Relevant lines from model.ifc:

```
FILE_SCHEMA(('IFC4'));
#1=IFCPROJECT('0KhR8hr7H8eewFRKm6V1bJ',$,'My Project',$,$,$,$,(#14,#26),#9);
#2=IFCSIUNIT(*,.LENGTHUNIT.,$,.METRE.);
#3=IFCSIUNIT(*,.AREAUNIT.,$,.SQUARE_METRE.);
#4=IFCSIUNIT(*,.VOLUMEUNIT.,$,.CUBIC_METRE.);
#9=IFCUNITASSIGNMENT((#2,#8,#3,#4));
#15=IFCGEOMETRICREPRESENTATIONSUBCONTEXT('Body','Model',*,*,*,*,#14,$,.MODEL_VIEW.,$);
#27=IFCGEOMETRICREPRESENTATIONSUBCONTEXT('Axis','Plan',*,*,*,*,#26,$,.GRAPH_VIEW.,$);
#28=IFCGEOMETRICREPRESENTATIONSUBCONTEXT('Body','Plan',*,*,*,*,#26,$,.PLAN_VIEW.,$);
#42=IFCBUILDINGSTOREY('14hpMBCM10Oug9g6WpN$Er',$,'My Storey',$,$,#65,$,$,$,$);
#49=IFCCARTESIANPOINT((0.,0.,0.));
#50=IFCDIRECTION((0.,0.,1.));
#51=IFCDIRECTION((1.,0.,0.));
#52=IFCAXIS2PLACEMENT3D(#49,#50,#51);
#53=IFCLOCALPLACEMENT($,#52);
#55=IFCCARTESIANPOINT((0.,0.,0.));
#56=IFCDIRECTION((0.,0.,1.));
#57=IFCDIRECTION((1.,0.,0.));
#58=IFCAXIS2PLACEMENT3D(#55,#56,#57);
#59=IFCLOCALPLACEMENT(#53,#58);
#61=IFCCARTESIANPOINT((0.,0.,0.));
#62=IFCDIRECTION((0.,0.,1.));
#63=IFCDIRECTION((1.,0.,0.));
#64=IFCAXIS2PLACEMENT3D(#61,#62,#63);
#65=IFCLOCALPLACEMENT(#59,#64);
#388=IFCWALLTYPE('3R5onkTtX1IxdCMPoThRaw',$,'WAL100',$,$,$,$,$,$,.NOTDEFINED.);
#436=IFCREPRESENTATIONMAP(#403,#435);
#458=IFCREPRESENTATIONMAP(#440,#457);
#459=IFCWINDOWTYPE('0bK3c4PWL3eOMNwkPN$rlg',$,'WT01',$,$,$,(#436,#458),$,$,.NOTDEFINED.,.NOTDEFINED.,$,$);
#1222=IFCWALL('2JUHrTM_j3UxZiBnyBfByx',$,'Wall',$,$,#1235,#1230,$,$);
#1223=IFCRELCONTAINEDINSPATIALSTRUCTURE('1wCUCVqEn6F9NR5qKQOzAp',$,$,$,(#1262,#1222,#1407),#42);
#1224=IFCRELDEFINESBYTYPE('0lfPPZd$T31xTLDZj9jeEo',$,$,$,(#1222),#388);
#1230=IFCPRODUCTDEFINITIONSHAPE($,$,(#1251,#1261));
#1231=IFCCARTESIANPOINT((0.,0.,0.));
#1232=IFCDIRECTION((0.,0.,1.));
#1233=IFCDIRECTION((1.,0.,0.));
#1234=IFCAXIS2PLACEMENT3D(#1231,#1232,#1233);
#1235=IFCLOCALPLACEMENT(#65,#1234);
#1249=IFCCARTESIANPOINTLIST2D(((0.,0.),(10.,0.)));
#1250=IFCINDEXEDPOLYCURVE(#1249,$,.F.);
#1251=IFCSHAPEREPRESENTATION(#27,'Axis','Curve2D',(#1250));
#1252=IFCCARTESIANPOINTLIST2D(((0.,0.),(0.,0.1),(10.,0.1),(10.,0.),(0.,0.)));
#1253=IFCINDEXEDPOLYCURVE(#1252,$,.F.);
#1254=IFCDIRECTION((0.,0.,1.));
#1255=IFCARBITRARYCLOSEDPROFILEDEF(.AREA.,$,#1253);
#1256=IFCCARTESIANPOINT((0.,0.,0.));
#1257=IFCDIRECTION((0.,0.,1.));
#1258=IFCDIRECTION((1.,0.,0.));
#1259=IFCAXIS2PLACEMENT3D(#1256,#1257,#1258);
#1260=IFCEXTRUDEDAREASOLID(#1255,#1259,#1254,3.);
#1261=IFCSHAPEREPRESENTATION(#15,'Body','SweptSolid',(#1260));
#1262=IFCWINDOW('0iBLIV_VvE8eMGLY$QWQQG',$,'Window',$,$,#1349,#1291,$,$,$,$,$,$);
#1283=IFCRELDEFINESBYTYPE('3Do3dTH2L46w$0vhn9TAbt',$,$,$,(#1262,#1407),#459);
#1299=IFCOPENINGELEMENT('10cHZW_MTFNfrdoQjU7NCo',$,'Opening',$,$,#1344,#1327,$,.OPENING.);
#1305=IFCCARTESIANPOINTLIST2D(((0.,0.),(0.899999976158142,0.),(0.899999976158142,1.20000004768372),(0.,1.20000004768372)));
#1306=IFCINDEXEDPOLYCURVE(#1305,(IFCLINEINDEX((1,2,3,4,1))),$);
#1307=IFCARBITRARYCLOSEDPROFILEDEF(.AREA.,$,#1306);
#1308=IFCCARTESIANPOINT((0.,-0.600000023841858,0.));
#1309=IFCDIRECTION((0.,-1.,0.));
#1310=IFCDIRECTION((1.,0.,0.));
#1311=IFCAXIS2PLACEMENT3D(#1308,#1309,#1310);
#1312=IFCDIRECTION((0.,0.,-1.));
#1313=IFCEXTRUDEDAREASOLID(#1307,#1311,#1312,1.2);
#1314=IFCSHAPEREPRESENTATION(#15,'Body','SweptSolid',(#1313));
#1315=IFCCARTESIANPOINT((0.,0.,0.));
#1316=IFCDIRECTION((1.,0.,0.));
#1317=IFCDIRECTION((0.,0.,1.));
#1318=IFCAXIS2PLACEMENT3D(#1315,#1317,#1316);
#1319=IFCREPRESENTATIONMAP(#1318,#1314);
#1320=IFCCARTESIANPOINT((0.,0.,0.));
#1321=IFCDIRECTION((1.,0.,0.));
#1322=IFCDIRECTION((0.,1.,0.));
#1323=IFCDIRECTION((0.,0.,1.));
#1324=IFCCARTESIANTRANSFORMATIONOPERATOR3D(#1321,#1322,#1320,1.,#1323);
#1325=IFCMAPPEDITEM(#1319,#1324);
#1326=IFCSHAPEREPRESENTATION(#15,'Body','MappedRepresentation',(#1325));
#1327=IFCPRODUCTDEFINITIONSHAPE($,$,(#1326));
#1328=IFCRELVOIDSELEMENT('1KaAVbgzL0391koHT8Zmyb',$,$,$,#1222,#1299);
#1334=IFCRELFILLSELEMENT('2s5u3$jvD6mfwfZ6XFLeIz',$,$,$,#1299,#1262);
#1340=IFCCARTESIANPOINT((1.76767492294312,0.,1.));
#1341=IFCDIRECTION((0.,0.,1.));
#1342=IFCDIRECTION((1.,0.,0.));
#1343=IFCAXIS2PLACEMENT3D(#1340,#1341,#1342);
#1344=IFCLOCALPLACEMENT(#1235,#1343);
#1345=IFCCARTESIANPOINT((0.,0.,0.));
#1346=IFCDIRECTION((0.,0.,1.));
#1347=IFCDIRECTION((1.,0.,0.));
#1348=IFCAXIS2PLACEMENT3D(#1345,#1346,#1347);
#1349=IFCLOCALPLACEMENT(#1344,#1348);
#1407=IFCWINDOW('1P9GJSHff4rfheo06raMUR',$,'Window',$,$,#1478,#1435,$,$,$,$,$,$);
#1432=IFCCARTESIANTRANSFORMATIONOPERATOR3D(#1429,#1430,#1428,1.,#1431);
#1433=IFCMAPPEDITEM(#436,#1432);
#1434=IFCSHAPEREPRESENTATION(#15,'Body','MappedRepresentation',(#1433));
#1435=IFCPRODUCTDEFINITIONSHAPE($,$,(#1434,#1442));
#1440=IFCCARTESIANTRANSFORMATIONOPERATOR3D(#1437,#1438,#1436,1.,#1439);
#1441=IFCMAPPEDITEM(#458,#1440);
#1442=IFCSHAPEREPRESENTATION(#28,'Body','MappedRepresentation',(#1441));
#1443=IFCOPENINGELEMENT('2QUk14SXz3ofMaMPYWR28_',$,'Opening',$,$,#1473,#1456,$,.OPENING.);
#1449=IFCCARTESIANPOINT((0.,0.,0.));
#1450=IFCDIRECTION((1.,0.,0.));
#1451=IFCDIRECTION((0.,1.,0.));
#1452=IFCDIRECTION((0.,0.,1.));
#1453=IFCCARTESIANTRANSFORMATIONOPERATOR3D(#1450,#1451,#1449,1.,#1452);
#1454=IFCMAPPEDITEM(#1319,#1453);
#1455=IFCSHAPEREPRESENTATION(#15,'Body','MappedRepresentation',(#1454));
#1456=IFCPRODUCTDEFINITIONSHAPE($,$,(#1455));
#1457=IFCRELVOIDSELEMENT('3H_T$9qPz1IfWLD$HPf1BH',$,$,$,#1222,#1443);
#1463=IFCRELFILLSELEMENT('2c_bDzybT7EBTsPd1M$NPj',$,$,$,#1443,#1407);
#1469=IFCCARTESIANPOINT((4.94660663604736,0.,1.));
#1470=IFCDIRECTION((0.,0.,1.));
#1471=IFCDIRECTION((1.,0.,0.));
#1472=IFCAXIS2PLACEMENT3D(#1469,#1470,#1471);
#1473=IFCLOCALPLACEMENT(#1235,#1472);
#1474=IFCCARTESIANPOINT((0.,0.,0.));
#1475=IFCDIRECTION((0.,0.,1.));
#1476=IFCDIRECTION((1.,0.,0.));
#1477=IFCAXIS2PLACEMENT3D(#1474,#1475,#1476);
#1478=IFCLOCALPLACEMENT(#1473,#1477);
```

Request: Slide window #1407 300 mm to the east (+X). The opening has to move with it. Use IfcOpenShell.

```python
import ifcopenshell
import ifcopenshell.api.geometry
import ifcopenshell.util.placement

model = ifcopenshell.open("model.ifc")

window = model.by_id(1407)
opening = window.FillsVoids[0].RelatingOpeningElement
wall = opening.VoidsElements[0].RelatingBuildingElement

wall_matrix = ifcopenshell.util.placement.get_local_placement(wall.ObjectPlacement)
shift = wall_matrix[:3, 0] * 0.3
before = ifcopenshell.util.placement.get_local_placement(window.ObjectPlacement)[:3, 3].copy()

# The window is placed relative to its opening, so it follows when the opening moves.
matrix = ifcopenshell.util.placement.get_local_placement(opening.ObjectPlacement)
matrix[:3, 3] += shift
ifcopenshell.api.geometry.edit_object_placement(
    model, product=opening, matrix=matrix, is_si=False, should_transform_children=True
)

after = ifcopenshell.util.placement.get_local_placement(window.ObjectPlacement)[:3, 3]
print("window moved by", (after - before).round(3) + 0.0)

model.write("model_updated.ifc")
```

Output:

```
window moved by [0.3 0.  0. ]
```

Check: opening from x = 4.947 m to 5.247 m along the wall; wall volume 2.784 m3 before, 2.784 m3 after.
